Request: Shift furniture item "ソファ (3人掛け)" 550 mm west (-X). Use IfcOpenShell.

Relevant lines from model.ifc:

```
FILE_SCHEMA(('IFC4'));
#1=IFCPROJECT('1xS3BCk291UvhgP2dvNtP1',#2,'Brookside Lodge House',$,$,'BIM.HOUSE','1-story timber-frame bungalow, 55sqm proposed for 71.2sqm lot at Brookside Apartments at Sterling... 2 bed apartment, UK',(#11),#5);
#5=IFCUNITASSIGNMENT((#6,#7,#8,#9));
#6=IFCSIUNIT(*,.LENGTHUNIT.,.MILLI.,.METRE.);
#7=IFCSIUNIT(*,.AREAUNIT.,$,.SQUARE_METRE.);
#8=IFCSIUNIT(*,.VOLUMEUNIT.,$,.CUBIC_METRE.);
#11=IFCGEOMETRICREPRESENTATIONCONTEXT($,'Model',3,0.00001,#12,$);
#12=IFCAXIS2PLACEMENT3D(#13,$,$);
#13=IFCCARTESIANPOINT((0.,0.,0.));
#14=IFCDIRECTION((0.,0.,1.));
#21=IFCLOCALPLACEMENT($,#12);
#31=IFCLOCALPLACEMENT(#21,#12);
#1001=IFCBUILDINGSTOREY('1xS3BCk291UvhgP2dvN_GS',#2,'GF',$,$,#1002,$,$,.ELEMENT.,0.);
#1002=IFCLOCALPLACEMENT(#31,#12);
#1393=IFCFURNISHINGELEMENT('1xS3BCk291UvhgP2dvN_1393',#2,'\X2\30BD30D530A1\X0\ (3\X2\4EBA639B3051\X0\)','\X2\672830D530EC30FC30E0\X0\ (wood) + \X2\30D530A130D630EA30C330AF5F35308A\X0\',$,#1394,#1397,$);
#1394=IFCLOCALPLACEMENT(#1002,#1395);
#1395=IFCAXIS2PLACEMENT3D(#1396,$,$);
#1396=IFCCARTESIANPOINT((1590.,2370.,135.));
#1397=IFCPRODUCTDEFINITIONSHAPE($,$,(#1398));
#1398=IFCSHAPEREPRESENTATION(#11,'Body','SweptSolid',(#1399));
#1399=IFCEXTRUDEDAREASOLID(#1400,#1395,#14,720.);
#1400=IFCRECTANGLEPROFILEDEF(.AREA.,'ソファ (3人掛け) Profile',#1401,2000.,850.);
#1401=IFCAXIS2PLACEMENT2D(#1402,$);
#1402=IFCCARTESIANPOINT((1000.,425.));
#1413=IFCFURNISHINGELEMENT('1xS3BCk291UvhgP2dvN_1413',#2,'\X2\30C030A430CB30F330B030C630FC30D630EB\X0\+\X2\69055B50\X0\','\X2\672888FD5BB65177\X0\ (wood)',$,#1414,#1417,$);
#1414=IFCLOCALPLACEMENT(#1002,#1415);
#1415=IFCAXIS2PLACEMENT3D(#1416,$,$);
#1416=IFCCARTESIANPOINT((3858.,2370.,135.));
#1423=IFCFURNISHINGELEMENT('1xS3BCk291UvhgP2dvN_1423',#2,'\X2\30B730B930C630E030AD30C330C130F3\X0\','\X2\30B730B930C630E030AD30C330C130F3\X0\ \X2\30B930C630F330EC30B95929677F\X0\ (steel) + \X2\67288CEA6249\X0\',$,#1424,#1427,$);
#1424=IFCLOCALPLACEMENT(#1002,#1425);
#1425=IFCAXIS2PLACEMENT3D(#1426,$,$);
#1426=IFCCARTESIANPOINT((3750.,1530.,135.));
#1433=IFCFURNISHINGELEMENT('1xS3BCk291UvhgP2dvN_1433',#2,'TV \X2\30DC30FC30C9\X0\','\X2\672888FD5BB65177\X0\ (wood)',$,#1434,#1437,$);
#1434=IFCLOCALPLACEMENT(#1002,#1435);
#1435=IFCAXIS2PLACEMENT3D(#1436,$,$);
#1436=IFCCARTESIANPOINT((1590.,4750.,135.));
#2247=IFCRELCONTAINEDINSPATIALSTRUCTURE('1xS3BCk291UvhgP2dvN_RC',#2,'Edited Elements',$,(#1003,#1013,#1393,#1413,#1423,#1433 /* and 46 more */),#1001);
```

```python
import ifcopenshell
import ifcopenshell.api.geometry
import ifcopenshell.util.placement
import ifcopenshell.util.unit

model = ifcopenshell.open("model.ifc")
unit_scale = ifcopenshell.util.unit.calculate_unit_scale(model)

item = model.by_guid("1xS3BCk291UvhgP2dvN_1393")
matrix = ifcopenshell.util.placement.get_local_placement(item.ObjectPlacement)
matrix[0, 3] -= 0.55 / unit_scale
ifcopenshell.api.geometry.edit_object_placement(model, product=item, matrix=matrix, is_si=False)

print(ifcopenshell.util.placement.get_local_placement(item.ObjectPlacement).round(3) + 0.0)

model.write("model_edited.ifc")
```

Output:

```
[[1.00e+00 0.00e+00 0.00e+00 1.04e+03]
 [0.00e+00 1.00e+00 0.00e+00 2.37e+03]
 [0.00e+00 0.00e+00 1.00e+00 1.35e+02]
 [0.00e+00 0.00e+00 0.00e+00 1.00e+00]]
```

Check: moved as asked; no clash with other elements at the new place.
